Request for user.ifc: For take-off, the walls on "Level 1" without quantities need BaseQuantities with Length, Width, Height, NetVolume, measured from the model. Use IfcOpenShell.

First a look at what the model holds.

```python
import ifcopenshell
import ifcopenshell.util.element
import ifcopenshell.util.unit

model = ifcopenshell.open("user.ifc")
print(model.schema)
for unit_type in ("LENGTHUNIT", "AREAUNIT", "VOLUMEUNIT"):
    print(unit_type, ifcopenshell.util.unit.calculate_unit_scale(model, unit_type))
storey = next(s for s in model.by_type("IfcBuildingStorey") if s.Name == "Level 1")
walls = [e for e in ifcopenshell.util.element.get_decomposition(storey) if e.is_a("IfcWall")]
for e in sorted(walls, key=lambda e: e.id()):
    print(e.id(), e.is_a(), e.Name, list(ifcopenshell.util.element.get_psets(e, qtos_only=True)), sep=" | ")
```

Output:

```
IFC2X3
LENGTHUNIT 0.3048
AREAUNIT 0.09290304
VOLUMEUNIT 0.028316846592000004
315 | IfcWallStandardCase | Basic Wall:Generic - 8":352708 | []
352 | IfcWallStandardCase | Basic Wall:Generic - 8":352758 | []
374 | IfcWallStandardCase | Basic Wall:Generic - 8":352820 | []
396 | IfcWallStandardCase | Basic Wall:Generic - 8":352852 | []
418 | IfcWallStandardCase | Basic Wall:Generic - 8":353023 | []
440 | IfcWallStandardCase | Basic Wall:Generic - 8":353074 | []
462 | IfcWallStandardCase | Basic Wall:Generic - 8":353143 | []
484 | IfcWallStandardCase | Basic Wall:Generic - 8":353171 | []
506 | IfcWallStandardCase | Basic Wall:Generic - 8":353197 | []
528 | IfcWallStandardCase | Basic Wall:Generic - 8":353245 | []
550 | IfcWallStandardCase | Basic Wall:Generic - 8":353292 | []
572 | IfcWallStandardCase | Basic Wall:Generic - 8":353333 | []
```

```python
import ifcopenshell
import ifcopenshell.api.pset
import ifcopenshell.geom
import ifcopenshell.util.element
import ifcopenshell.util.shape
import ifcopenshell.util.unit

model = ifcopenshell.open("user.ifc")
unit_scale = ifcopenshell.util.unit.calculate_unit_scale(model)
volume_scale = ifcopenshell.util.unit.calculate_unit_scale(model, "VOLUMEUNIT")
settings = ifcopenshell.geom.settings()

storey = next(s for s in model.by_type("IfcBuildingStorey") if s.Name == "Level 1")
walls = [e for e in ifcopenshell.util.element.get_decomposition(storey) if e.is_a("IfcWall")]

for e in sorted(walls, key=lambda e: e.id()):
    if ifcopenshell.util.element.get_psets(e, qtos_only=True, should_inherit=False):
        continue
    # Geometry comes back in metres, in the element's own axes.
    shape = ifcopenshell.geom.create_shape(settings, e)
    values = {
        "Length": ifcopenshell.util.shape.get_x(shape.geometry) / unit_scale,
        "Width": ifcopenshell.util.shape.get_y(shape.geometry) / unit_scale,
        "Height": ifcopenshell.util.shape.get_z(shape.geometry) / unit_scale,
        "NetVolume": ifcopenshell.util.shape.get_volume(shape.geometry) / volume_scale,
    }
    qto = ifcopenshell.api.pset.add_qto(model, product=e, name="BaseQuantities")
    ifcopenshell.api.pset.edit_qto(model, qto=qto, properties=values)
    print(e.id(), {k: round(v, 3) for k, v in values.items()})

model.write("user_v2.ifc")
```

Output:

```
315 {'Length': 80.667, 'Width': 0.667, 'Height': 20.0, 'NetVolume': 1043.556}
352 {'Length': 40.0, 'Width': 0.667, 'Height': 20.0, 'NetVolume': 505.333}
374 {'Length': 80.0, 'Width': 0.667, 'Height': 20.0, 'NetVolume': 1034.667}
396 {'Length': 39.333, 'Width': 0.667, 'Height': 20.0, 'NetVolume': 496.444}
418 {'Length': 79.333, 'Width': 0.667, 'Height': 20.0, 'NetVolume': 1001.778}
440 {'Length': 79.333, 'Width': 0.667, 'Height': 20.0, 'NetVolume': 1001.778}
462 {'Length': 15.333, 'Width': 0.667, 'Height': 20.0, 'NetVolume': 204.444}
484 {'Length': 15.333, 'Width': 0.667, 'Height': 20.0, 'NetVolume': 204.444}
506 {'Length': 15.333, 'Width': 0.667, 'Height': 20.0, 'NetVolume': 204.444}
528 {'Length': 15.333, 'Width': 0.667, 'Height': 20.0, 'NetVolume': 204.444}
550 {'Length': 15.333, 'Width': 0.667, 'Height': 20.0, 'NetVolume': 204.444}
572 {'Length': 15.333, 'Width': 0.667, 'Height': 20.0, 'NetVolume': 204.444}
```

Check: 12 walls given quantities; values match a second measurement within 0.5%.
